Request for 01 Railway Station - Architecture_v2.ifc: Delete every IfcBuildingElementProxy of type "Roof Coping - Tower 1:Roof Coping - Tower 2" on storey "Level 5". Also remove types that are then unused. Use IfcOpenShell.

First a look at what the model holds.

```python
import ifcopenshell
import ifcopenshell.util.element

model = ifcopenshell.open("01 Railway Station - Architecture_v2.ifc")
print(model.schema)
storey = next(s for s in model.by_type("IfcBuildingStorey") if s.Name == "Level 5")
proxies = [e for e in ifcopenshell.util.element.get_decomposition(storey) if e.is_a("IfcBuildingElementProxy")]
seen = {}
for e in proxies:
    element_type = ifcopenshell.util.element.get_type(e)
    name = element_type.Name if element_type not in (None, e) else None
    seen[name] = seen.get(name, 0) + 1
for name, count in sorted(seen.items(), key=str):
    print(count, "x", name)
```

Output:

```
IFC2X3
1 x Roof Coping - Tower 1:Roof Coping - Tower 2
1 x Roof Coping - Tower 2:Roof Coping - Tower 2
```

```python
import ifcopenshell
import ifcopenshell.api.root
import ifcopenshell.util.element

model = ifcopenshell.open("01 Railway Station - Architecture_v2.ifc")

storey = next(s for s in model.by_type("IfcBuildingStorey") if s.Name == "Level 5")
proxies = [e for e in ifcopenshell.util.element.get_decomposition(storey) if e.is_a("IfcBuildingElementProxy")]
targets = [e for e in proxies if (t := ifcopenshell.util.element.get_type(e)) not in (None, e) and t.Name == "Roof Coping - Tower 1:Roof Coping - Tower 2"]
types = {ifcopenshell.util.element.get_type(e) for e in targets} - {None, *targets}

for e in targets:
    ifcopenshell.api.root.remove_product(model, product=e)
print(len(targets), "removed")

unused = [t for t in types if not ifcopenshell.util.element.get_types(t)]
for t in unused:
    ifcopenshell.api.root.remove_product(model, product=t)
print(len(unused), "unused types removed")

model.write("01 Railway Station - Architecture_v2-out.ifc")
```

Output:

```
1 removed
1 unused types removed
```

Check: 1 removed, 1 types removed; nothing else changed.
